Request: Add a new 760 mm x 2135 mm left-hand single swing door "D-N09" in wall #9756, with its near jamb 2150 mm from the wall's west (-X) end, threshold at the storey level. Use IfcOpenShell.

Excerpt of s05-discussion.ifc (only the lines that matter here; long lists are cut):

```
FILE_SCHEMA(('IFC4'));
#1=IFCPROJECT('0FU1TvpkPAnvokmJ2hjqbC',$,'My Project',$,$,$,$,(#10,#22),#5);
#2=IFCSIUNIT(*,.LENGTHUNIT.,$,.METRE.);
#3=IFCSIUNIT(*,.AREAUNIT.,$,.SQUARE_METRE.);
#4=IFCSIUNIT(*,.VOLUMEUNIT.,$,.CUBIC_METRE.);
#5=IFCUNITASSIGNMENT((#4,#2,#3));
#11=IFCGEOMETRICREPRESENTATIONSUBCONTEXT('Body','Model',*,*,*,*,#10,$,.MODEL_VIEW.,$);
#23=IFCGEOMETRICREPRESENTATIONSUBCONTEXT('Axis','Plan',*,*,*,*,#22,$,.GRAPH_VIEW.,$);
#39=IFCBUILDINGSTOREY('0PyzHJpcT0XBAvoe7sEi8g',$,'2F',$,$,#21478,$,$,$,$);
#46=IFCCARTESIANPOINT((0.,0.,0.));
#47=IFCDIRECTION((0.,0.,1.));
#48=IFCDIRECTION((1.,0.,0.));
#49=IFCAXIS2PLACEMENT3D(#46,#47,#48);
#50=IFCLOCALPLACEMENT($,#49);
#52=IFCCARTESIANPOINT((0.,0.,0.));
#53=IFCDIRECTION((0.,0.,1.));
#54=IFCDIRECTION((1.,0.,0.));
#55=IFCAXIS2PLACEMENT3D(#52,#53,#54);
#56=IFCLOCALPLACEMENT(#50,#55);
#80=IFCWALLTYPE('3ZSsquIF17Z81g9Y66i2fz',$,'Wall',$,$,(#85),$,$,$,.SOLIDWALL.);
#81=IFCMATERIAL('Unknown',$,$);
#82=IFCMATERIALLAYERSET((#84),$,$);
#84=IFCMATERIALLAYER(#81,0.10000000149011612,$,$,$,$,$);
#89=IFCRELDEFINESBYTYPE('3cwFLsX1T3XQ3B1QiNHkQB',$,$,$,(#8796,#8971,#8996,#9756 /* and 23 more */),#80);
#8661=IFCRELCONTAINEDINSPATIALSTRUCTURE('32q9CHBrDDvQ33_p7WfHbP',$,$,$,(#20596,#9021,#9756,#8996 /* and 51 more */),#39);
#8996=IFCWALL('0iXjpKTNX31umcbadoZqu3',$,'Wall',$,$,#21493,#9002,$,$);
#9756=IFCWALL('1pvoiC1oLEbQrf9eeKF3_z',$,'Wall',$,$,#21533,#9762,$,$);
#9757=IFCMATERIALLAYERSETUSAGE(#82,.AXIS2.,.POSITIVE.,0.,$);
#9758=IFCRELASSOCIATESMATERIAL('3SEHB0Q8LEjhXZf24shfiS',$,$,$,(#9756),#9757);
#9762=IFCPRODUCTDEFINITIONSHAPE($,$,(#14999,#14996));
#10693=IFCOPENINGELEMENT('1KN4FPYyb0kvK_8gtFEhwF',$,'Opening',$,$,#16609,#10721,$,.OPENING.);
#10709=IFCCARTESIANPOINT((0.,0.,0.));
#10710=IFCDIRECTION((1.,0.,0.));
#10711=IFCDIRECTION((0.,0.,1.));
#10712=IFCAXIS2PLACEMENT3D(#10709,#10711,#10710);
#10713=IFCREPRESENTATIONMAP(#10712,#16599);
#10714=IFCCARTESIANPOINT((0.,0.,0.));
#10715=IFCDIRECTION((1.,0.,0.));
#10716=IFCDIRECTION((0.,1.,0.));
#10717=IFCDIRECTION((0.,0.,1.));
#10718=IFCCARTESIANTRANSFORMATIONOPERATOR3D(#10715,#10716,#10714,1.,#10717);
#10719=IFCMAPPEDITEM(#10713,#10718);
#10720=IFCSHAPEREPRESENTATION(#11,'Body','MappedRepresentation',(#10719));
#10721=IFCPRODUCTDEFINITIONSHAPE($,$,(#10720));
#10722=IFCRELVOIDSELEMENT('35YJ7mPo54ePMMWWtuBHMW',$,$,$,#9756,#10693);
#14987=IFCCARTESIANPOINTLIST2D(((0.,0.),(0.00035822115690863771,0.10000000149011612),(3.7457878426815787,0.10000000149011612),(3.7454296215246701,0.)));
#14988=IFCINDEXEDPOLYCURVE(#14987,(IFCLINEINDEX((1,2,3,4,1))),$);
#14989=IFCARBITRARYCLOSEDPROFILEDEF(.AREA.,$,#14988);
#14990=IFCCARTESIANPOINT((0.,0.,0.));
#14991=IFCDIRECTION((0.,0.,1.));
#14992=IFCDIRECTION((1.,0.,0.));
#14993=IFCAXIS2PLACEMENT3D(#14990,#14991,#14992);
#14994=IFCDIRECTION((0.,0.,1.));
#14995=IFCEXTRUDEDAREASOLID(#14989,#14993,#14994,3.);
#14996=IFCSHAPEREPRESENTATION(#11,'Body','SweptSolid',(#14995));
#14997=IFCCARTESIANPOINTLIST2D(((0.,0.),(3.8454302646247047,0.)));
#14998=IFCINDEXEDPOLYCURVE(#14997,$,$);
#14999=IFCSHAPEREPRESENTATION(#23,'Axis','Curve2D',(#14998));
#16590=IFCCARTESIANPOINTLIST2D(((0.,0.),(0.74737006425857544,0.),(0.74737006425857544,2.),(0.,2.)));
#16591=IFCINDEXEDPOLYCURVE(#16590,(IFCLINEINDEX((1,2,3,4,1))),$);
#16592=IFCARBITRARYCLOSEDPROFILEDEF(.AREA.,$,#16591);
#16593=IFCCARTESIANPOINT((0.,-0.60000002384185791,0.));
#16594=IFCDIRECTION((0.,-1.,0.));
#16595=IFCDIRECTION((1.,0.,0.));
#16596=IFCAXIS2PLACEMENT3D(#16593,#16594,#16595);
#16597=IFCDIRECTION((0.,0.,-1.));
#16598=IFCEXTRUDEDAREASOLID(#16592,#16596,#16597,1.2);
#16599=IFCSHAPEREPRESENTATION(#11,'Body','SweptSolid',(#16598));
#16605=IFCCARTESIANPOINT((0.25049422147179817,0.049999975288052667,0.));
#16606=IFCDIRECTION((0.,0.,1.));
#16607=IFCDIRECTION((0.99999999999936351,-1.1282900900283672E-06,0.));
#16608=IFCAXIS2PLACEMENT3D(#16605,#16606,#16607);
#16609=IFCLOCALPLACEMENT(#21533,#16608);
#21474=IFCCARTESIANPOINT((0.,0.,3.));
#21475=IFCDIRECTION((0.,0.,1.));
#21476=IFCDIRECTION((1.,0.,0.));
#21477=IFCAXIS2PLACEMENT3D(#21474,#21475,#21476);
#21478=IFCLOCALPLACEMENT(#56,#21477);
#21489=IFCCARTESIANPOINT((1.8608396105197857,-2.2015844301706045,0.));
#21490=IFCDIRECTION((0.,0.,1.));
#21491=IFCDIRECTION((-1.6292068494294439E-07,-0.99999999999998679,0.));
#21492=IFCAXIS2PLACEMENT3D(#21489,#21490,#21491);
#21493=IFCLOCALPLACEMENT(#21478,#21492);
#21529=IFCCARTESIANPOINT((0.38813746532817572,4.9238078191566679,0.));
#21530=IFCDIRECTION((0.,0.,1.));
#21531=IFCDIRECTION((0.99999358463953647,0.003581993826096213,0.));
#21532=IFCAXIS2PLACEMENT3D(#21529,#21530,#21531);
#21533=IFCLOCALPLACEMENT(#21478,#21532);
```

```python
import numpy as np
import ifcopenshell
import ifcopenshell.api.feature
import ifcopenshell.api.geometry
import ifcopenshell.api.root
import ifcopenshell.api.spatial
import ifcopenshell.geom
import ifcopenshell.util.element
import ifcopenshell.util.placement
import ifcopenshell.util.representation
import ifcopenshell.util.shape
import ifcopenshell.util.unit

model = ifcopenshell.open("s05-discussion.ifc")
unit_scale = ifcopenshell.util.unit.calculate_unit_scale(model)
settings = ifcopenshell.geom.settings()


def volume(element):
    """Net volume in cubic metres, openings subtracted."""
    shape = ifcopenshell.geom.create_shape(settings, element)
    return ifcopenshell.util.shape.get_volume(shape.geometry)


wall = model.by_guid("1pvoiC1oLEbQrf9eeKF3_z")
storey = ifcopenshell.util.element.get_container(wall, ifc_class="IfcBuildingStorey")
context = ifcopenshell.util.representation.get_context(model, "Model", "Body", "MODEL_VIEW")
before = volume(wall)

width, height, from_end, sill = 0.76, 2.135, 2.15, 0.0  # metres

# The wall runs along its own X axis, and the end named is its -X end.
wall_shape = ifcopenshell.geom.create_shape(settings, wall)
x, y, z = ifcopenshell.util.shape.get_vertices(wall_shape.geometry).T
start = x.min() + from_end
face, thickness = float(y.min()), float(y.max() - y.min())
wall_matrix = ifcopenshell.util.placement.get_local_placement(wall.ObjectPlacement)
level = ifcopenshell.util.placement.get_local_placement(storey.ObjectPlacement)[2, 3]


def in_wall(x, y):
    """Placement at x, y metres in the wall's axes, at sill height."""
    matrix = wall_matrix.copy()
    matrix[:, 3] = wall_matrix @ np.array([x / unit_scale, y / unit_scale, 0.0, 1.0])
    matrix[2, 3] = level + sill / unit_scale
    return matrix


# Opening: a box that overshoots both wall faces by 50 mm.
opening = ifcopenshell.api.root.create_entity(model, ifc_class="IfcOpeningElement", predefined_type="OPENING")
box = ifcopenshell.api.geometry.add_wall_representation(
    model, context=context, length=width, height=height, thickness=thickness + 0.1
)
ifcopenshell.api.geometry.assign_representation(model, product=opening, representation=box)
ifcopenshell.api.geometry.edit_object_placement(model, product=opening, matrix=in_wall(start, face - 0.05), is_si=False)
ifcopenshell.api.feature.add_feature(model, feature=opening, element=wall)

door = ifcopenshell.api.root.create_entity(model, ifc_class="IfcDoor", name="D-N09", predefined_type="DOOR")
door.OverallWidth, door.OverallHeight = width / unit_scale, height / unit_scale
door.OperationType = "SINGLE_SWING_LEFT"
body = ifcopenshell.api.geometry.add_door_representation(
    model,
    context=context,
    overall_width=door.OverallWidth,
    overall_height=door.OverallHeight,
    operation_type="SINGLE_SWING_LEFT",
    lining_properties={"LiningDepth": thickness / unit_scale, "ThresholdDepth": thickness / unit_scale},
)
ifcopenshell.api.geometry.assign_representation(model, product=door, representation=body)
ifcopenshell.api.spatial.assign_container(model, products=[door], relating_structure=storey)
ifcopenshell.api.feature.add_filling(model, opening=opening, element=door)

# The lining spans the wall, so the door starts at the wall face.
ifcopenshell.api.geometry.edit_object_placement(model, product=door, matrix=in_wall(start, face), is_si=False)

after = volume(wall)

print(f"wall volume {before:.3f} -> {after:.3f} m3")

model.write("s05-discussion-out.ifc")
```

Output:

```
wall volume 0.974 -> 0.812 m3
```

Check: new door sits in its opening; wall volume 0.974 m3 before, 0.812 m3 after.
